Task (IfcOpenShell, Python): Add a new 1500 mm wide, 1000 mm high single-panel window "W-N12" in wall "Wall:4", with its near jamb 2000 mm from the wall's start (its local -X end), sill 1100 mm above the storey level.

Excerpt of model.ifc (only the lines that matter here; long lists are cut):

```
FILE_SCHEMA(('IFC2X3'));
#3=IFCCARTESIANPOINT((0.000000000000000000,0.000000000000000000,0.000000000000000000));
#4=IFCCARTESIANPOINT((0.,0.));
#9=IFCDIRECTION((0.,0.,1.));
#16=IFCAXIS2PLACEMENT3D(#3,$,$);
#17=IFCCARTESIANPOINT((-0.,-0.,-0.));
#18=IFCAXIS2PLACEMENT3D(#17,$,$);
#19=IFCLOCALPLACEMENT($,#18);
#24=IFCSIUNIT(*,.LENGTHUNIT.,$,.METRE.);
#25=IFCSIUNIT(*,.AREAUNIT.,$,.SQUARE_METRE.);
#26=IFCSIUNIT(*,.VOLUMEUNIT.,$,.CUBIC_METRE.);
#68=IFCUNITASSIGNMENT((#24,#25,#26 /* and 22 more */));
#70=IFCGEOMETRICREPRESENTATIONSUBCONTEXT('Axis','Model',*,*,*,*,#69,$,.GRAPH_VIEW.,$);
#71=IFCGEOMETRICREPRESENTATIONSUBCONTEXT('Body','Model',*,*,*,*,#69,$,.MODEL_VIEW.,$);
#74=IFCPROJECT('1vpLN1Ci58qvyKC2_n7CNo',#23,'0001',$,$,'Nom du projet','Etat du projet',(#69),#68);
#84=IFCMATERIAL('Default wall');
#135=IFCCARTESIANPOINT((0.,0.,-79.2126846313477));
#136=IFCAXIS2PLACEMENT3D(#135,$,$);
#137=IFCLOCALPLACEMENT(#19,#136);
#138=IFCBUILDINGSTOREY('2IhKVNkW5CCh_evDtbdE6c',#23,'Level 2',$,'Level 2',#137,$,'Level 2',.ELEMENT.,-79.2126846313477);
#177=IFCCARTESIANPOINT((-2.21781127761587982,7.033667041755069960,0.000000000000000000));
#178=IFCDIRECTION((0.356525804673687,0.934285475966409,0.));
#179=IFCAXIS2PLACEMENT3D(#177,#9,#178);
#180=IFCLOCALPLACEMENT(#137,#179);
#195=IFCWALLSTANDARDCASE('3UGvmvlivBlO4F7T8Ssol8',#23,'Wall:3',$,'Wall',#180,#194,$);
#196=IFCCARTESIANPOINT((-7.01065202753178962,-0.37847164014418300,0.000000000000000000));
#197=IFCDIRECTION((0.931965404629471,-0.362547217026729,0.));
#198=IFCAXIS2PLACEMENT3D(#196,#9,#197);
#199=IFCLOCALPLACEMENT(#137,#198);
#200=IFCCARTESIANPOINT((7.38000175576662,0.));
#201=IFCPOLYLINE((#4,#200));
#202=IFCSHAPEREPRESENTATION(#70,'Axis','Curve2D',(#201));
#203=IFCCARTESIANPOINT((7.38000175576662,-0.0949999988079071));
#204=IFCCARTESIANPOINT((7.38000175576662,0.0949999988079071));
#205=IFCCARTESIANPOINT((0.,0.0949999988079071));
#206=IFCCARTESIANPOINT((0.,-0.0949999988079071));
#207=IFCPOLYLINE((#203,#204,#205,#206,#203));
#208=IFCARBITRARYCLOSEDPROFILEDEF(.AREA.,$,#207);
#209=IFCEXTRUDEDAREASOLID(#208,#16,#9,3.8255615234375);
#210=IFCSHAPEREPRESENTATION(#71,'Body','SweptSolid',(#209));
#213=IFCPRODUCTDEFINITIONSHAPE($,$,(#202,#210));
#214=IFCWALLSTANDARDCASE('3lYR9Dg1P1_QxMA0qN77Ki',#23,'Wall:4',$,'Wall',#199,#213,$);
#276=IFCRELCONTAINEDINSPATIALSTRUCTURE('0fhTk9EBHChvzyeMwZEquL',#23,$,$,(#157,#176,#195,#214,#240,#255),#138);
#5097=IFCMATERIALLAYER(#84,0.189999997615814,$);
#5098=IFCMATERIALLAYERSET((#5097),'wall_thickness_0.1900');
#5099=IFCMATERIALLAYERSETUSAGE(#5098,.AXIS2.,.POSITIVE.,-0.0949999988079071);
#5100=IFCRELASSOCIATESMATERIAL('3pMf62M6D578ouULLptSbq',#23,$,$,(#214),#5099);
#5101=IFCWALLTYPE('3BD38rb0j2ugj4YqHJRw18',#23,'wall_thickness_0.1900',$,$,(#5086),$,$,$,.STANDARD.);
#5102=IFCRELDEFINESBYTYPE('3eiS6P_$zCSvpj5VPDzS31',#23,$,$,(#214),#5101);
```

```python
import numpy as np
import ifcopenshell
import ifcopenshell.api.feature
import ifcopenshell.api.geometry
import ifcopenshell.api.root
import ifcopenshell.api.spatial
import ifcopenshell.api.type
import ifcopenshell.geom
import ifcopenshell.util.element
import ifcopenshell.util.placement
import ifcopenshell.util.representation
import ifcopenshell.util.shape
import ifcopenshell.util.unit

model = ifcopenshell.open("model.ifc")
unit_scale = ifcopenshell.util.unit.calculate_unit_scale(model)
settings = ifcopenshell.geom.settings()


def volume(element):
    """Net volume in cubic metres, openings subtracted."""
    shape = ifcopenshell.geom.create_shape(settings, element)
    return ifcopenshell.util.shape.get_volume(shape.geometry)


wall = model.by_id(214)
storey = ifcopenshell.util.element.get_container(wall, ifc_class="IfcBuildingStorey")
context = ifcopenshell.util.representation.get_context(model, "Model", "Body", "MODEL_VIEW")
before = volume(wall)

width, height, from_end, sill = 1.5, 1, 2, 1.1  # metres

# The wall runs along its own X axis, and the end named is its -X end.
wall_shape = ifcopenshell.geom.create_shape(settings, wall)
x, y, z = ifcopenshell.util.shape.get_vertices(wall_shape.geometry).T
start = x.min() + from_end
face, thickness = float(y.min()), float(y.max() - y.min())
wall_matrix = ifcopenshell.util.placement.get_local_placement(wall.ObjectPlacement)
level = ifcopenshell.util.placement.get_local_placement(storey.ObjectPlacement)[2, 3]


def in_wall(x, y):
    """Placement at x, y metres in the wall's axes, at sill height."""
    matrix = wall_matrix.copy()
    matrix[:, 3] = wall_matrix @ np.array([x / unit_scale, y / unit_scale, 0.0, 1.0])
    matrix[2, 3] = level + sill / unit_scale
    return matrix


# Opening: a box that overshoots both wall faces by 50 mm.
opening = ifcopenshell.api.root.create_entity(model, ifc_class="IfcOpeningElement")
box = ifcopenshell.api.geometry.add_wall_representation(
    model, context=context, length=width, height=height, thickness=thickness + 0.1
)
ifcopenshell.api.geometry.assign_representation(model, product=opening, representation=box)
ifcopenshell.api.geometry.edit_object_placement(model, product=opening, matrix=in_wall(start, face - 0.05), is_si=False)
ifcopenshell.api.feature.add_feature(model, feature=opening, element=wall)

window = ifcopenshell.api.root.create_entity(model, ifc_class="IfcWindow", name="W-N12")
window.OverallWidth, window.OverallHeight = width / unit_scale, height / unit_scale
body = ifcopenshell.api.geometry.add_window_representation(
    model,
    context=context,
    overall_width=window.OverallWidth,
    overall_height=window.OverallHeight,
    partition_type="SINGLE_PANEL",
)
ifcopenshell.api.geometry.assign_representation(model, product=window, representation=body)
ifcopenshell.api.spatial.assign_container(model, products=[window], relating_structure=storey)
fills = ifcopenshell.api.feature.add_filling(model, opening=opening, element=window)
fills.OwnerHistory = window.OwnerHistory  # required in IFC2X3

# IFC2X3 keeps the operation on the window style.
style = ifcopenshell.api.root.create_entity(model, ifc_class="IfcWindowStyle", name="W-N12")
style.OperationType, style.ConstructionType = "SINGLE_PANEL", "NOTDEFINED"
style.ParameterTakesPrecedence = style.Sizeable = False
ifcopenshell.api.type.assign_type(model, related_objects=[window], relating_type=style)

# Centre the window in the wall's thickness.
ifcopenshell.api.geometry.edit_object_placement(model, product=window, matrix=in_wall(start, face), is_si=False)
window_shape = ifcopenshell.geom.create_shape(settings, window)
depth = ifcopenshell.util.shape.get_vertices(window_shape.geometry)[:, 1]
offset = face + thickness / 2 - (depth.min() + depth.max()) / 2
ifcopenshell.api.geometry.edit_object_placement(model, product=window, matrix=in_wall(start, offset), is_si=False)

after = volume(wall)

print(f"wall volume {before:.3f} -> {after:.3f} m3")

model.write("model-out.ifc")
```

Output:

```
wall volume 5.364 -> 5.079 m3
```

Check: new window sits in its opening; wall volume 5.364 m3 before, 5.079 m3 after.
